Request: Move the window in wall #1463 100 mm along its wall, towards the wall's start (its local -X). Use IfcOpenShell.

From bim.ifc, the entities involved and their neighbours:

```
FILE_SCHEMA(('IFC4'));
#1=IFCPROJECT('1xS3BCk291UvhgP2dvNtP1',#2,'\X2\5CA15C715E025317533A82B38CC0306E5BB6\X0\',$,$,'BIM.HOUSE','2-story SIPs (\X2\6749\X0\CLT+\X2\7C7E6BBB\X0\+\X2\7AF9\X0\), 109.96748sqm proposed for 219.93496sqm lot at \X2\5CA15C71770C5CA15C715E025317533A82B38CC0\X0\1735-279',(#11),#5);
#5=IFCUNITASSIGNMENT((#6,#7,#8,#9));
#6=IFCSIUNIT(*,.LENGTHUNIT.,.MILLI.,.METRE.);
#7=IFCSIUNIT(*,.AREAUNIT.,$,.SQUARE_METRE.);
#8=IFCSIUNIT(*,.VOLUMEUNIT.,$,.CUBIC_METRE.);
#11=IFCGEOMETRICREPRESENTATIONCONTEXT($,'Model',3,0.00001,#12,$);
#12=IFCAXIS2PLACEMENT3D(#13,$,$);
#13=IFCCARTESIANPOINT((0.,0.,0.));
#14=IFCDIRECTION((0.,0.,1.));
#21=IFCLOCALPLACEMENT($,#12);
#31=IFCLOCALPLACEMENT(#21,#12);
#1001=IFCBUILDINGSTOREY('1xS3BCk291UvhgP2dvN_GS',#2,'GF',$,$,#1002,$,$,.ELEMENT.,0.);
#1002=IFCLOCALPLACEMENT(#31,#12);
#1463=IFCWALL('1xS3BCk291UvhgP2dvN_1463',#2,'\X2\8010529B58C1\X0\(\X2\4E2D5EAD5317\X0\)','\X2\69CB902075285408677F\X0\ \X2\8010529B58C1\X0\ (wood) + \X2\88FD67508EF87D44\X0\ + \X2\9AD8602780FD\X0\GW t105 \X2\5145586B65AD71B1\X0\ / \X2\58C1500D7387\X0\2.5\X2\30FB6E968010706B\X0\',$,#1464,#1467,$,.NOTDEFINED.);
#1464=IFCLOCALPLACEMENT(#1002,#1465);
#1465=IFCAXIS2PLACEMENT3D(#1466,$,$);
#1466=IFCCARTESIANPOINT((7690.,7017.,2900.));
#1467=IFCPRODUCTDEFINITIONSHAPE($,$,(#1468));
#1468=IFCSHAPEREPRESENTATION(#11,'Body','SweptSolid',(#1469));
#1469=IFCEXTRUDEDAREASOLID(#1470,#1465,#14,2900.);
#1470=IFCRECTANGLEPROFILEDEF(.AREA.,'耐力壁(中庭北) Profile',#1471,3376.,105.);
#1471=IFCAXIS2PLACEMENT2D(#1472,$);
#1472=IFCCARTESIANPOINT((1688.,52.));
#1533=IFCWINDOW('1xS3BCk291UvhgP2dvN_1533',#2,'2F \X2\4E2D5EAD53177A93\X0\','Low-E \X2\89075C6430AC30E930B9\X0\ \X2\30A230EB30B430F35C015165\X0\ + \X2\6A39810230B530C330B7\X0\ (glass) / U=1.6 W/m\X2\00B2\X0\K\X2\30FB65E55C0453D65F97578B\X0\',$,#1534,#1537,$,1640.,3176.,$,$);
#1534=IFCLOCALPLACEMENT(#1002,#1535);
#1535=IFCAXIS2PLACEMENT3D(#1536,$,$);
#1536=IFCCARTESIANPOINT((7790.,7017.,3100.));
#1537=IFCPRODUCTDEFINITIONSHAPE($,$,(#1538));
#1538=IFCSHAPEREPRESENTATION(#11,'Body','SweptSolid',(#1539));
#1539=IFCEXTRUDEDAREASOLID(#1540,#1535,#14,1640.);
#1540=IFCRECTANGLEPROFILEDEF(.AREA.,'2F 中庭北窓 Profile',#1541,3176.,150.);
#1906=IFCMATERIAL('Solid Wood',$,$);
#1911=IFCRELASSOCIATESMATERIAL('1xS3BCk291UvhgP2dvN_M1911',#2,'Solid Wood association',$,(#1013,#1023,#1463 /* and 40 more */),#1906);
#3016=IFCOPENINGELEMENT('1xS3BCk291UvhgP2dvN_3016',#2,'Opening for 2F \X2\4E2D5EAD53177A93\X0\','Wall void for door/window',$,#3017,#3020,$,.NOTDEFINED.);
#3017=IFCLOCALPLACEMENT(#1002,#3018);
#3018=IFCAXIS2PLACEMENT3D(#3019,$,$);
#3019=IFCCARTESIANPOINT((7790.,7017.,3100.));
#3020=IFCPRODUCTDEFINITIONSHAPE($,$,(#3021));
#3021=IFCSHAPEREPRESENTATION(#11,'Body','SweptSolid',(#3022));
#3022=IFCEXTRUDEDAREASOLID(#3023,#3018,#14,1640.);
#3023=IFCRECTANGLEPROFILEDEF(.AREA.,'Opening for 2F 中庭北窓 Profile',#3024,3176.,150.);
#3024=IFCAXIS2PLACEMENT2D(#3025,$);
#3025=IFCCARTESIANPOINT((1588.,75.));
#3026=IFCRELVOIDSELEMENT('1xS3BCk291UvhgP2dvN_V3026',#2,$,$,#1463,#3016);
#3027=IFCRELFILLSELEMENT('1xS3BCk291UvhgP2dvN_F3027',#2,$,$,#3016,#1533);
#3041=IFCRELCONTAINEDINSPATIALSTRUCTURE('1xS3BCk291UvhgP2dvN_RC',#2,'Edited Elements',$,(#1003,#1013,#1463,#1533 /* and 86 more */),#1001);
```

```python
import ifcopenshell
import ifcopenshell.api.geometry
import ifcopenshell.util.placement

model = ifcopenshell.open("bim.ifc")

window = model.by_guid("1xS3BCk291UvhgP2dvN_1533")
opening = window.FillsVoids[0].RelatingOpeningElement
wall = opening.VoidsElements[0].RelatingBuildingElement

wall_matrix = ifcopenshell.util.placement.get_local_placement(wall.ObjectPlacement)
shift = wall_matrix[:3, 0] * -100.0
before = ifcopenshell.util.placement.get_local_placement(window.ObjectPlacement)[:3, 3].copy()

# The window is not placed relative to its opening, so move both.
for product in (opening, window):
    matrix = ifcopenshell.util.placement.get_local_placement(product.ObjectPlacement)
    matrix[:3, 3] += shift
    ifcopenshell.api.geometry.edit_object_placement(model, product=product, matrix=matrix, is_si=False)

after = ifcopenshell.util.placement.get_local_placement(window.ObjectPlacement)[:3, 3]
print("window moved by", (after - before).round(3) + 0.0)

model.write("bim_rev.ifc")
```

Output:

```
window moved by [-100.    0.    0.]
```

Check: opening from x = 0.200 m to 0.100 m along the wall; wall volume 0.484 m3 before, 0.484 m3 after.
